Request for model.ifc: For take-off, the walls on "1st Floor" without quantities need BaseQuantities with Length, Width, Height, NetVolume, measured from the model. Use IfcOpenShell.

First a look at what the model holds.

```python
import ifcopenshell
import ifcopenshell.util.element
import ifcopenshell.util.unit

model = ifcopenshell.open("model.ifc")
print(model.schema)
for unit_type in ("LENGTHUNIT", "AREAUNIT", "VOLUMEUNIT"):
    print(unit_type, ifcopenshell.util.unit.calculate_unit_scale(model, unit_type))
storey = next(s for s in model.by_type("IfcBuildingStorey") if s.Name == "1st Floor")
walls = [e for e in ifcopenshell.util.element.get_decomposition(storey) if e.is_a("IfcWall")]
for e in sorted(walls, key=lambda e: e.id()):
    print(e.id(), e.is_a(), e.Name, list(ifcopenshell.util.element.get_psets(e, qtos_only=True)), sep=" | ")
```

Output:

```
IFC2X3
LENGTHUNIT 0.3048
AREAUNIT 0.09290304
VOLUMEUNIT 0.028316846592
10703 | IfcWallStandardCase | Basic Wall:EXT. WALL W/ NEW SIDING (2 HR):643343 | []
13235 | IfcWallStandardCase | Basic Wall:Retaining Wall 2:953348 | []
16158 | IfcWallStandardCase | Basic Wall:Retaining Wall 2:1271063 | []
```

```python
import ifcopenshell
import ifcopenshell.api.pset
import ifcopenshell.geom
import ifcopenshell.util.element
import ifcopenshell.util.shape
import ifcopenshell.util.unit

model = ifcopenshell.open("model.ifc")
unit_scale = ifcopenshell.util.unit.calculate_unit_scale(model)
volume_scale = ifcopenshell.util.unit.calculate_unit_scale(model, "VOLUMEUNIT")
settings = ifcopenshell.geom.settings()

storey = next(s for s in model.by_type("IfcBuildingStorey") if s.Name == "1st Floor")
walls = [e for e in ifcopenshell.util.element.get_decomposition(storey) if e.is_a("IfcWall")]

for e in sorted(walls, key=lambda e: e.id()):
    if ifcopenshell.util.element.get_psets(e, qtos_only=True, should_inherit=False):
        continue
    # Geometry comes back in metres, in the element's own axes.
    shape = ifcopenshell.geom.create_shape(settings, e)
    values = {
        "Length": ifcopenshell.util.shape.get_x(shape.geometry) / unit_scale,
        "Width": ifcopenshell.util.shape.get_y(shape.geometry) / unit_scale,
        "Height": ifcopenshell.util.shape.get_z(shape.geometry) / unit_scale,
        "NetVolume": ifcopenshell.util.shape.get_volume(shape.geometry) / volume_scale,
    }
    qto = ifcopenshell.api.pset.add_qto(model, product=e, name="BaseQuantities")
    ifcopenshell.api.pset.edit_qto(model, qto=qto, properties=values)
    print(e.id(), {k: round(v, 3) for k, v in values.items()})

model.write("model_updated.ifc")
```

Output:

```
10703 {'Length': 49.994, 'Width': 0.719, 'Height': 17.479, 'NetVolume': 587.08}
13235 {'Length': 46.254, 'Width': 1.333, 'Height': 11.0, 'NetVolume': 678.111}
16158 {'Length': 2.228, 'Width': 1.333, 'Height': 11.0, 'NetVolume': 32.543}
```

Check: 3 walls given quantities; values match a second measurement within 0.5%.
